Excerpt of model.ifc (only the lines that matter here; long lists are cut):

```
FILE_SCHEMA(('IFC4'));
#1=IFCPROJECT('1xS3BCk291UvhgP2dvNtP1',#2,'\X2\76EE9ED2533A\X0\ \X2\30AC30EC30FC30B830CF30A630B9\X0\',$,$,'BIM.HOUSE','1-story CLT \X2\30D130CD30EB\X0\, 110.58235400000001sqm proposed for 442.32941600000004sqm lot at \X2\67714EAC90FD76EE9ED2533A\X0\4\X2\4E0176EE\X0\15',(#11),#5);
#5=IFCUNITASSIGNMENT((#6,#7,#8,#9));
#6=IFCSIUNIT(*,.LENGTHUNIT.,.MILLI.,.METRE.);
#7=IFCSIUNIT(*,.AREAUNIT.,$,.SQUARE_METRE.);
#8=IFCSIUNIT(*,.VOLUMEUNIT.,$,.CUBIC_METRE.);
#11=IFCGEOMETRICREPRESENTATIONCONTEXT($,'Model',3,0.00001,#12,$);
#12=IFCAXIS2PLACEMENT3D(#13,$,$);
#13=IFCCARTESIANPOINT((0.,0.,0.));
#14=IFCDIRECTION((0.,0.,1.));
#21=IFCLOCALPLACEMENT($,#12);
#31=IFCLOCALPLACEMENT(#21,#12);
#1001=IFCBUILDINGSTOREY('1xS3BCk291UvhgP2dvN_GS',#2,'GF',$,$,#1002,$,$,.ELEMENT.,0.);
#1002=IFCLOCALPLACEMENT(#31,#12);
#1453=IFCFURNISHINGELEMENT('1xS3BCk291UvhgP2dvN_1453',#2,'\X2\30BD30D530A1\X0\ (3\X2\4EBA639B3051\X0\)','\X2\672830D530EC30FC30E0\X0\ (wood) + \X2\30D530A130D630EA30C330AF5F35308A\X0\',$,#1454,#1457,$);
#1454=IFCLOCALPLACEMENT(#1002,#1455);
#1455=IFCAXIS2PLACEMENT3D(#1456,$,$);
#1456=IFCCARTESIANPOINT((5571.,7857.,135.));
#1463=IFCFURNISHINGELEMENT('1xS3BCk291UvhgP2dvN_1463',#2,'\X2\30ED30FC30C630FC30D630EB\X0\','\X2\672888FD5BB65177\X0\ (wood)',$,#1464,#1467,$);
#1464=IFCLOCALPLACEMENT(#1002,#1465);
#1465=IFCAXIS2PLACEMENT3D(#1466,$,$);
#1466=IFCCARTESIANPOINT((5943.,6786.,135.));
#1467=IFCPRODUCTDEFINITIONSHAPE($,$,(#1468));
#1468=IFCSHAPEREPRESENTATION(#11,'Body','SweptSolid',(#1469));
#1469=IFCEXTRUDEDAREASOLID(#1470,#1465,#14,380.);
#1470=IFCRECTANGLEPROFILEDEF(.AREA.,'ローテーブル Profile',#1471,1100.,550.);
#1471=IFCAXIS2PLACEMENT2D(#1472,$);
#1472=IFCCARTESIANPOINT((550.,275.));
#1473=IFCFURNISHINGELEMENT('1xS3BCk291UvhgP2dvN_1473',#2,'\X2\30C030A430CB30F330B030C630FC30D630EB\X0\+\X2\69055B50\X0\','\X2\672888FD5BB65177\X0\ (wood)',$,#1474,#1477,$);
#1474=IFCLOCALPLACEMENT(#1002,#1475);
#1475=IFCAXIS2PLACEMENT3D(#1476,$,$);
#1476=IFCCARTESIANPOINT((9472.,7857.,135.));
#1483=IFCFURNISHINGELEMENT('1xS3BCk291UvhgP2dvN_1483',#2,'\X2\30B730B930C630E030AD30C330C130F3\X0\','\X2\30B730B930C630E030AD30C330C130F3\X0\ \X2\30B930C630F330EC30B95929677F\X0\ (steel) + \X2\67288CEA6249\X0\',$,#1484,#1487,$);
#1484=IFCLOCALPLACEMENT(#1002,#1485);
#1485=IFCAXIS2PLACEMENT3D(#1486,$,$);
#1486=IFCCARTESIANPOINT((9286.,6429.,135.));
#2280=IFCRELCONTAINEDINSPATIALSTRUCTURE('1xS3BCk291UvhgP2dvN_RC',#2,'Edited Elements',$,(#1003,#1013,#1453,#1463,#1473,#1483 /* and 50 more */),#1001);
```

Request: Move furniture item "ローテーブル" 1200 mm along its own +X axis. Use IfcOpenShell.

```python
import ifcopenshell
import ifcopenshell.api.geometry
import ifcopenshell.util.placement

model = ifcopenshell.open("model.ifc")

item = model.by_guid("1xS3BCk291UvhgP2dvN_1463")
matrix = ifcopenshell.util.placement.get_local_placement(item.ObjectPlacement)
matrix[:3, 3] += matrix[:3, 0] * 1200.0
ifcopenshell.api.geometry.edit_object_placement(model, product=item, matrix=matrix, is_si=False)

print(ifcopenshell.util.placement.get_local_placement(item.ObjectPlacement).round(3) + 0.0)

model.write("model_rev.ifc")
```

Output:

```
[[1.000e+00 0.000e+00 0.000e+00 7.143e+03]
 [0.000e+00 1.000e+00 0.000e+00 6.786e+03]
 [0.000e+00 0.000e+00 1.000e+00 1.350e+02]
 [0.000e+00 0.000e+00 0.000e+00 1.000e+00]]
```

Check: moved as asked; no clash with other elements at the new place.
